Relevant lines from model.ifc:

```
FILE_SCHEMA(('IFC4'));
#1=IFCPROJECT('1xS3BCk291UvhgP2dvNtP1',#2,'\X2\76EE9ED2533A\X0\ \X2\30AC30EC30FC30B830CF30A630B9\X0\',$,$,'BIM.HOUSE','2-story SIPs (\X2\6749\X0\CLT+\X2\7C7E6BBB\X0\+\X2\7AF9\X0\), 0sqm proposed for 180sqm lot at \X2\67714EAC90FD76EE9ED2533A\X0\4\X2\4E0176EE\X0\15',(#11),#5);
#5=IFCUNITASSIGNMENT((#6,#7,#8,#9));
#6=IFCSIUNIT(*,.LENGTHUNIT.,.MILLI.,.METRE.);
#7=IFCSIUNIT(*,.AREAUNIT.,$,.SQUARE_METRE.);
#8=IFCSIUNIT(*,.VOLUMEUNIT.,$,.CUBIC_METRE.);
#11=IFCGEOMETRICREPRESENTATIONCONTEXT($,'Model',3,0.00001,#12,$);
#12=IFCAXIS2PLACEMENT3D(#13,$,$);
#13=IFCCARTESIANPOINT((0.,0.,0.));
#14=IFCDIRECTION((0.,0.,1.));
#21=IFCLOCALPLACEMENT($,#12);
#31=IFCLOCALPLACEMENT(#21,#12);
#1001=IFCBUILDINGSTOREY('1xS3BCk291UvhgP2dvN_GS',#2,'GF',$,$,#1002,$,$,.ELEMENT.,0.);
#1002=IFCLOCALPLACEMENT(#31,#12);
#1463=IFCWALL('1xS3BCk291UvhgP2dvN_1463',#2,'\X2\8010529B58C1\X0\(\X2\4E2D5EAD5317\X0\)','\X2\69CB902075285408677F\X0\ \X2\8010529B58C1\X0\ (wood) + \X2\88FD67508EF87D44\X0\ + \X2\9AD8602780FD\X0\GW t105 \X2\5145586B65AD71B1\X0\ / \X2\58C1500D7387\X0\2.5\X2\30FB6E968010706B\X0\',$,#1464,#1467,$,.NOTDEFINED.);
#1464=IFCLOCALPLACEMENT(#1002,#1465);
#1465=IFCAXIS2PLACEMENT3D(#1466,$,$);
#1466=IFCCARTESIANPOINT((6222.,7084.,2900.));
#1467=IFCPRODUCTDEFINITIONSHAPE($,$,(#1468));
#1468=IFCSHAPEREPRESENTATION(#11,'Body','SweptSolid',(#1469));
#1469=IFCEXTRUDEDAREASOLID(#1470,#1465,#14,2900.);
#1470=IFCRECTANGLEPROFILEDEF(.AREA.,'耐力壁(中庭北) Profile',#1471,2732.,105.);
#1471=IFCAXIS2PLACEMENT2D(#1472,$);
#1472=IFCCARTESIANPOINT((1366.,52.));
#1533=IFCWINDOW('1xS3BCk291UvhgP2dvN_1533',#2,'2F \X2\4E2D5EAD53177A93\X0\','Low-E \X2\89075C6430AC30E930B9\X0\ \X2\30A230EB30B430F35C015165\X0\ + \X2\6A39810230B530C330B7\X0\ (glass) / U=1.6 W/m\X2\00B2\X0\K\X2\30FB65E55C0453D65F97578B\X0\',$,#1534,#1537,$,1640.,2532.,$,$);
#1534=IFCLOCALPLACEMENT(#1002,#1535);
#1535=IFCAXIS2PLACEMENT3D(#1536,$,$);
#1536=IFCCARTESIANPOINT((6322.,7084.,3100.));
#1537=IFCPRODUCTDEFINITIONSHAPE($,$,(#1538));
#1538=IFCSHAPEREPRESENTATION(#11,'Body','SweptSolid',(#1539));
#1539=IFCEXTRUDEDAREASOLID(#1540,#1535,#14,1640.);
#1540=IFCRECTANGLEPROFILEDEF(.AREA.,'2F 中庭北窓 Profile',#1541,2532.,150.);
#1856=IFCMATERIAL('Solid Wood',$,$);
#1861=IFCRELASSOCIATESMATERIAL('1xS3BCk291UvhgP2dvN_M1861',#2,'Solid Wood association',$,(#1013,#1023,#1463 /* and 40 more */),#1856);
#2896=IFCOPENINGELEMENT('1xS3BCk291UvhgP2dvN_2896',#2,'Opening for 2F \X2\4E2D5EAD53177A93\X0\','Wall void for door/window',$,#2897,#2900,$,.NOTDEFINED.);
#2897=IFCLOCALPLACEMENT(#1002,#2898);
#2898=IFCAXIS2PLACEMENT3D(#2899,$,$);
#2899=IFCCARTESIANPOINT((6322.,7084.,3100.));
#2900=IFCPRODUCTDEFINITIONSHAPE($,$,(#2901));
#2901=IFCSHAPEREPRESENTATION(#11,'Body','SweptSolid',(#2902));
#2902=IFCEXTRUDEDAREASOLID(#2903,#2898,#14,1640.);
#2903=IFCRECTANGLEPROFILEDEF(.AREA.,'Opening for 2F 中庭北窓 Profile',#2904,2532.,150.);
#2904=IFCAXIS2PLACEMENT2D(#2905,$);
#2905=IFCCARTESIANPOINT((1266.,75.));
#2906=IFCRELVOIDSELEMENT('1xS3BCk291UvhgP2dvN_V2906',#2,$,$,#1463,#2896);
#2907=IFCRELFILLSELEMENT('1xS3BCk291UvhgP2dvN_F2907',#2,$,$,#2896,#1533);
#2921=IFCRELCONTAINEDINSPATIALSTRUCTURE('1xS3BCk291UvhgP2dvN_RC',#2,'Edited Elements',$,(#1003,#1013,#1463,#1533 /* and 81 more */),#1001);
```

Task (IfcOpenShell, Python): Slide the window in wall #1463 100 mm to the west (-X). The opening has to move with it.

```python
import ifcopenshell
import ifcopenshell.api.geometry
import ifcopenshell.util.placement

model = ifcopenshell.open("model.ifc")

window = model.by_guid("1xS3BCk291UvhgP2dvN_1533")
opening = window.FillsVoids[0].RelatingOpeningElement
wall = opening.VoidsElements[0].RelatingBuildingElement

wall_matrix = ifcopenshell.util.placement.get_local_placement(wall.ObjectPlacement)
shift = wall_matrix[:3, 0] * -100.0
before = ifcopenshell.util.placement.get_local_placement(window.ObjectPlacement)[:3, 3].copy()

# The window is not placed relative to its opening, so move both.
for product in (opening, window):
    matrix = ifcopenshell.util.placement.get_local_placement(product.ObjectPlacement)
    matrix[:3, 3] += shift
    ifcopenshell.api.geometry.edit_object_placement(model, product=product, matrix=matrix, is_si=False)

after = ifcopenshell.util.placement.get_local_placement(window.ObjectPlacement)[:3, 3]
print("window moved by", (after - before).round(3) + 0.0)

model.write("model_updated.ifc")
```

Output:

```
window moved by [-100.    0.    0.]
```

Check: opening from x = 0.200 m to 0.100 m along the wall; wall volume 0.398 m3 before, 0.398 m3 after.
